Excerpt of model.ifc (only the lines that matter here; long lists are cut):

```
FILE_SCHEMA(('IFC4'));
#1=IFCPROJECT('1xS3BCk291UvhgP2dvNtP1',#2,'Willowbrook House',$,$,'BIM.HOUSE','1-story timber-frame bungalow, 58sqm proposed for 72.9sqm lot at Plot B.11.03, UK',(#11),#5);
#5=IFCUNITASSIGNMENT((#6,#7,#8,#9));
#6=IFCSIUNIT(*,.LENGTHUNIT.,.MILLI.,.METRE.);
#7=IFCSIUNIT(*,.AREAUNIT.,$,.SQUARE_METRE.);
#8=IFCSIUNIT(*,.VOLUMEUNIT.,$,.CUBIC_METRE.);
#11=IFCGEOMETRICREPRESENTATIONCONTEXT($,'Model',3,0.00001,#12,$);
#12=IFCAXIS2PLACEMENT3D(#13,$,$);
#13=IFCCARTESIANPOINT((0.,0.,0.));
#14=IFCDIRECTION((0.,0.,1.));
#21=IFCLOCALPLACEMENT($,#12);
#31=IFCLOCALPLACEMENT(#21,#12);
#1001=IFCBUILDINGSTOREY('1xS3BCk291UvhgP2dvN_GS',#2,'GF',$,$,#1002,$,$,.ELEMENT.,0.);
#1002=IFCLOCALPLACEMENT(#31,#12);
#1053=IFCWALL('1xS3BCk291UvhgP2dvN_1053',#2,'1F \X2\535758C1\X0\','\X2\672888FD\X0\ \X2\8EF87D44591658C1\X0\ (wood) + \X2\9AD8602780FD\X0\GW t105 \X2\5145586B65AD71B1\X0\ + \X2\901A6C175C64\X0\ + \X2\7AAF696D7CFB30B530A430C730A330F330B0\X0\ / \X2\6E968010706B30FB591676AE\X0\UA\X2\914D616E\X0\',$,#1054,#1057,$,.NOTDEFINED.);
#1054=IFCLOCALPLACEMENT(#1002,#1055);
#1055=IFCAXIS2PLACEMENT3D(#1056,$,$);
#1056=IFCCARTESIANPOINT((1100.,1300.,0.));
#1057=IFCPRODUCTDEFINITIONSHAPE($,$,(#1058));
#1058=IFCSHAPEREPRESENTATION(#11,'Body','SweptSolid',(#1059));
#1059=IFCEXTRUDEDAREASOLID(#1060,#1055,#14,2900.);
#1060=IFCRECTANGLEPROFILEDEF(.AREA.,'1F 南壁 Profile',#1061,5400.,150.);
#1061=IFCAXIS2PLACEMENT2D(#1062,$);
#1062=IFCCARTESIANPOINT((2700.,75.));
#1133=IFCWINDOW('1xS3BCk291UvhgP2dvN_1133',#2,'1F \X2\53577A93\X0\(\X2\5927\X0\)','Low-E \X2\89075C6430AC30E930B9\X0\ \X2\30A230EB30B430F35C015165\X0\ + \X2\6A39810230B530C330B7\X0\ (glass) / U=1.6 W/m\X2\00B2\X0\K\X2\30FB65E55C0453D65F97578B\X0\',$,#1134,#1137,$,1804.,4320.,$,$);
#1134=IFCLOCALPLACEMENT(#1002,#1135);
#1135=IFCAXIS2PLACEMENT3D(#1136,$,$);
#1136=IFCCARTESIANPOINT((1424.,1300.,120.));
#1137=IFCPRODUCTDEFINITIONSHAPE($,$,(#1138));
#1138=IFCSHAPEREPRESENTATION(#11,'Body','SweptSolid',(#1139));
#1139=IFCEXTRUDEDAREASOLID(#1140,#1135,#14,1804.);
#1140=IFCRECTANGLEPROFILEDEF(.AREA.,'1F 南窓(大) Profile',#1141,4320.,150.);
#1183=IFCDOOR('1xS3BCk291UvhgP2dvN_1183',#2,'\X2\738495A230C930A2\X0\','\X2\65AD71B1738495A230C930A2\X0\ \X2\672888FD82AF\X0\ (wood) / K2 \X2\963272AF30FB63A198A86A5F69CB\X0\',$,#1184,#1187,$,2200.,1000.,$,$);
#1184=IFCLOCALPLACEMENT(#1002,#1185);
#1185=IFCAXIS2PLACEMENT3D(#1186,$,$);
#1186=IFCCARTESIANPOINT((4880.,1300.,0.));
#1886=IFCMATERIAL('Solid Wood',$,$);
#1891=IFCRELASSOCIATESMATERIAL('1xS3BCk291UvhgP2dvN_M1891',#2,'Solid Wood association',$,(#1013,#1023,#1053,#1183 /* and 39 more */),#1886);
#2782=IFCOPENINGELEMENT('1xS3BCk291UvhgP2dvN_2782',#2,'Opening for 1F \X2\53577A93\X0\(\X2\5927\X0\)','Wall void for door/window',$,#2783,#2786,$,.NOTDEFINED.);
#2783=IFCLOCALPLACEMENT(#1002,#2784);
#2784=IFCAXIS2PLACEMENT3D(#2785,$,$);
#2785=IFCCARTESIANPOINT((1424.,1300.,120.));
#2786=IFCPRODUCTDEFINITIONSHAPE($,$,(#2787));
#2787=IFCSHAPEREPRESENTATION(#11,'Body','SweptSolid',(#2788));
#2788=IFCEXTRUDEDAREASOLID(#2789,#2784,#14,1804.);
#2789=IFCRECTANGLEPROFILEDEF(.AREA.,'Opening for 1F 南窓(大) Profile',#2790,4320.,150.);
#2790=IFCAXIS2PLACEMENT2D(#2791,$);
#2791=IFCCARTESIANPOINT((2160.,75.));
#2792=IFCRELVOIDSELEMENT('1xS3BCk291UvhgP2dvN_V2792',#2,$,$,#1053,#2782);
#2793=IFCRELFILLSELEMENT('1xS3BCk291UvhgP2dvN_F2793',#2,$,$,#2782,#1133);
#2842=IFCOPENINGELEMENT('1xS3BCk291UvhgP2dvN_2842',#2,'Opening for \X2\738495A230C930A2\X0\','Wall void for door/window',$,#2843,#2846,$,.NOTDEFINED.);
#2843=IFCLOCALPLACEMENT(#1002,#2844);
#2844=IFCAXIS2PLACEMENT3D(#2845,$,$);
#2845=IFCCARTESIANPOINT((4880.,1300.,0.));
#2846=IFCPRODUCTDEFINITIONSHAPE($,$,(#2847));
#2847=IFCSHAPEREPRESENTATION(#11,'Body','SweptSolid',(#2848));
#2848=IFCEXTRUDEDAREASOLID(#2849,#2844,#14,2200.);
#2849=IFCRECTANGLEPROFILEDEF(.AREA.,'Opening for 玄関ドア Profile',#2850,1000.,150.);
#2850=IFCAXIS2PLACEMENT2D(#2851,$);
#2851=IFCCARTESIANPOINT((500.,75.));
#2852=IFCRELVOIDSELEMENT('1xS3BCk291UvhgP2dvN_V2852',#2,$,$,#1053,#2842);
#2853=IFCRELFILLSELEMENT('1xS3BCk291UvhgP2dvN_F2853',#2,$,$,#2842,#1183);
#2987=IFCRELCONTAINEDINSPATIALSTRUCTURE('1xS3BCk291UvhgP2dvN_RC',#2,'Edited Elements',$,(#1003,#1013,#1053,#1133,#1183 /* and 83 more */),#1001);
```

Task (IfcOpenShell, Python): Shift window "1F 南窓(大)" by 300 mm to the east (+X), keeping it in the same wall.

```python
import ifcopenshell
import ifcopenshell.api.geometry
import ifcopenshell.util.placement

model = ifcopenshell.open("model.ifc")

window = model.by_guid("1xS3BCk291UvhgP2dvN_1133")
opening = window.FillsVoids[0].RelatingOpeningElement
wall = opening.VoidsElements[0].RelatingBuildingElement

wall_matrix = ifcopenshell.util.placement.get_local_placement(wall.ObjectPlacement)
shift = wall_matrix[:3, 0] * 300.0
before = ifcopenshell.util.placement.get_local_placement(window.ObjectPlacement)[:3, 3].copy()

# The window is not placed relative to its opening, so move both.
for product in (opening, window):
    matrix = ifcopenshell.util.placement.get_local_placement(product.ObjectPlacement)
    matrix[:3, 3] += shift
    ifcopenshell.api.geometry.edit_object_placement(model, product=product, matrix=matrix, is_si=False)

after = ifcopenshell.util.placement.get_local_placement(window.ObjectPlacement)[:3, 3]
print("window moved by", (after - before).round(3) + 0.0)

model.write("model_v2.ifc")
```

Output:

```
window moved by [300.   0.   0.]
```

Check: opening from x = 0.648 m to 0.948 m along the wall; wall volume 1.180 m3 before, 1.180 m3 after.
